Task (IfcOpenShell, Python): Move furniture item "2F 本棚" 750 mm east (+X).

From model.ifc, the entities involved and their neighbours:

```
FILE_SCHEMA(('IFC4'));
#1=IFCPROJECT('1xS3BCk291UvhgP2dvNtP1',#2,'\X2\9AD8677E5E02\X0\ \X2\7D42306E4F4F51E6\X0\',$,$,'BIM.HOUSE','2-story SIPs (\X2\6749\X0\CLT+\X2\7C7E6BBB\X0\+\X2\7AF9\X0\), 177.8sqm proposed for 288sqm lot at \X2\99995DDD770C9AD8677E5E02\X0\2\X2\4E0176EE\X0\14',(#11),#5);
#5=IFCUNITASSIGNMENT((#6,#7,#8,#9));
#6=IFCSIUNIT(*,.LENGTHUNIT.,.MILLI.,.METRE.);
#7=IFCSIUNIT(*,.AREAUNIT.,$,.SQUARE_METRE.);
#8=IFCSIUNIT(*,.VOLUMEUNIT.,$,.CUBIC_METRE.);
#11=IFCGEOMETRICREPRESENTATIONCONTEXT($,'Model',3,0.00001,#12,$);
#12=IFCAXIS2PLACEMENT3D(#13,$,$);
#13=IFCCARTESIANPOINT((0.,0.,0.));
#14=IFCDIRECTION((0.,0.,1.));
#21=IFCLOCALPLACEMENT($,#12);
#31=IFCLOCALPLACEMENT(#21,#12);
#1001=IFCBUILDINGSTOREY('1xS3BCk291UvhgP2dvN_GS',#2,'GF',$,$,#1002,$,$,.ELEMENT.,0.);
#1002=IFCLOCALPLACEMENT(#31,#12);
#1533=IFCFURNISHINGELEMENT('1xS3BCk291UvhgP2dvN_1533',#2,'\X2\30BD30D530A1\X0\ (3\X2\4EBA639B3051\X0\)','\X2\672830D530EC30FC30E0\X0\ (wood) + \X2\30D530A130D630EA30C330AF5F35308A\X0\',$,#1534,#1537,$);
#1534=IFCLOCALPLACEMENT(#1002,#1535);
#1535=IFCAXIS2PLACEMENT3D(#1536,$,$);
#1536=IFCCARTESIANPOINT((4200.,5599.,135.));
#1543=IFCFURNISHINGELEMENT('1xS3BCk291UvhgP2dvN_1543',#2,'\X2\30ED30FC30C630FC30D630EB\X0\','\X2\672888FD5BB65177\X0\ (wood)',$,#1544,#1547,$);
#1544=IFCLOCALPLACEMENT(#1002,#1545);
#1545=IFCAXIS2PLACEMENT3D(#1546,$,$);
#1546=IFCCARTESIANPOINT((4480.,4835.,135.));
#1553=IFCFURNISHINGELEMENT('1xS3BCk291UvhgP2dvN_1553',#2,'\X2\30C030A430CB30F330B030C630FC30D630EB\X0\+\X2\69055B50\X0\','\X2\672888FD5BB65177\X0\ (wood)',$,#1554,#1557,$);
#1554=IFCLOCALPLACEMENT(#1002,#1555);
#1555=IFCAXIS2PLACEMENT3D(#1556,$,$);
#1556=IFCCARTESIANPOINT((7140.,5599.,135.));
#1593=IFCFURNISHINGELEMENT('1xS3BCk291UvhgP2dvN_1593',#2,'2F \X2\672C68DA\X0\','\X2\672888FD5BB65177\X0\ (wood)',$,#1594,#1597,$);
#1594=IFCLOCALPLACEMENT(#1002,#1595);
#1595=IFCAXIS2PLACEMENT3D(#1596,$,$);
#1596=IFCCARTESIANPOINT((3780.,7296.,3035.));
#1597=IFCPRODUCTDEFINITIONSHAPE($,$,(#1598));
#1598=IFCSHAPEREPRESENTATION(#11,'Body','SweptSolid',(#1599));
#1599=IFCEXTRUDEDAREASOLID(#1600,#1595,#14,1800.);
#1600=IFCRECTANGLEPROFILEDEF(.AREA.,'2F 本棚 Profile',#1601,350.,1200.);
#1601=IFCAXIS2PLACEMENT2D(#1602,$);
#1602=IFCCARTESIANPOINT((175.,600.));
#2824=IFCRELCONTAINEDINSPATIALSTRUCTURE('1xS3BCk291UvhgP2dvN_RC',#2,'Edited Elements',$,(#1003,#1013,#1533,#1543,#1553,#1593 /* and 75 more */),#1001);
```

```python
import ifcopenshell
import ifcopenshell.api.geometry
import ifcopenshell.util.placement
import ifcopenshell.util.unit

model = ifcopenshell.open("model.ifc")
unit_scale = ifcopenshell.util.unit.calculate_unit_scale(model)

item = model.by_id(1593)
matrix = ifcopenshell.util.placement.get_local_placement(item.ObjectPlacement)
matrix[0, 3] += 0.75 / unit_scale
ifcopenshell.api.geometry.edit_object_placement(model, product=item, matrix=matrix, is_si=False)

print(ifcopenshell.util.placement.get_local_placement(item.ObjectPlacement).round(3) + 0.0)

model.write("model_rev.ifc")
```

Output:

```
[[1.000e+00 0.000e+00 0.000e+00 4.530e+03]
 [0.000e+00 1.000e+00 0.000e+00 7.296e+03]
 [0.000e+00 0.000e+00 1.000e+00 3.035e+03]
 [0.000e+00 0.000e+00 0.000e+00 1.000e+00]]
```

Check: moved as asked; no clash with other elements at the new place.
